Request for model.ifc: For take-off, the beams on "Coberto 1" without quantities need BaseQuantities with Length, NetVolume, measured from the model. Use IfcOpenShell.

First a look at what the model holds.

```python
import ifcopenshell
import ifcopenshell.util.element
import ifcopenshell.util.unit

model = ifcopenshell.open("model.ifc")
print(model.schema)
for unit_type in ("LENGTHUNIT", "AREAUNIT", "VOLUMEUNIT"):
    print(unit_type, ifcopenshell.util.unit.calculate_unit_scale(model, unit_type))
storey = next(s for s in model.by_type("IfcBuildingStorey") if s.Name == "Coberto 1")
beams = [e for e in ifcopenshell.util.element.get_decomposition(storey) if e.is_a("IfcBeam")]
for e in sorted(beams, key=lambda e: e.id()):
    print(e.id(), e.is_a(), e.Name, list(ifcopenshell.util.element.get_psets(e, qtos_only=True)), sep=" | ")
```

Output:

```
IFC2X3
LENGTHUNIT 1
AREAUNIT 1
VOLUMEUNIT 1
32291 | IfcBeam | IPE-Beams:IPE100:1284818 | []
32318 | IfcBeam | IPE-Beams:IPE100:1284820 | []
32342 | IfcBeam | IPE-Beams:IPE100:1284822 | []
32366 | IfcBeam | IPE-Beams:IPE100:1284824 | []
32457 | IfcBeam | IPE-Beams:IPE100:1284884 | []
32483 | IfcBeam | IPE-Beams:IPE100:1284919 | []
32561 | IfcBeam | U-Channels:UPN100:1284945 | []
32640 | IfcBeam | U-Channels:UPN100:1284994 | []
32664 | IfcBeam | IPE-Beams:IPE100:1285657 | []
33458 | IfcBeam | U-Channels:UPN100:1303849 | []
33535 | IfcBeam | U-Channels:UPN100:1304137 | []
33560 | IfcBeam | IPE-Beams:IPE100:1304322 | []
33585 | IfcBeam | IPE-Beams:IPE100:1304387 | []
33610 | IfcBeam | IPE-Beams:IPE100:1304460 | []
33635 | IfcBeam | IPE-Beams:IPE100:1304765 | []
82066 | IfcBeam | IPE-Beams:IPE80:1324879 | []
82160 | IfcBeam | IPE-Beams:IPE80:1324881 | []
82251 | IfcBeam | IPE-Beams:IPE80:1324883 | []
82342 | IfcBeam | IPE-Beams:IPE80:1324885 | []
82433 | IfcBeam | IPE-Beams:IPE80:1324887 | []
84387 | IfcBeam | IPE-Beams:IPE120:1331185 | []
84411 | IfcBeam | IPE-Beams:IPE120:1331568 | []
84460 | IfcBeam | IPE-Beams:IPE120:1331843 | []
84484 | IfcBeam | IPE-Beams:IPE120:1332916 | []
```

```python
import ifcopenshell
import ifcopenshell.api.pset
import ifcopenshell.geom
import ifcopenshell.util.element
import ifcopenshell.util.shape
import ifcopenshell.util.unit

model = ifcopenshell.open("model.ifc")
unit_scale = ifcopenshell.util.unit.calculate_unit_scale(model)
volume_scale = ifcopenshell.util.unit.calculate_unit_scale(model, "VOLUMEUNIT")
settings = ifcopenshell.geom.settings()

storey = next(s for s in model.by_type("IfcBuildingStorey") if s.Name == "Coberto 1")
beams = [e for e in ifcopenshell.util.element.get_decomposition(storey) if e.is_a("IfcBeam")]

for e in sorted(beams, key=lambda e: e.id()):
    if ifcopenshell.util.element.get_psets(e, qtos_only=True, should_inherit=False):
        continue
    # Geometry comes back in metres, in the element's own axes.
    shape = ifcopenshell.geom.create_shape(settings, e)
    values = {
        "Length": ifcopenshell.util.shape.get_max_xyz(shape.geometry) / unit_scale,
        "NetVolume": ifcopenshell.util.shape.get_volume(shape.geometry) / volume_scale,
    }
    qto = ifcopenshell.api.pset.add_qto(model, product=e, name="BaseQuantities")
    ifcopenshell.api.pset.edit_qto(model, qto=qto, properties=values)
    print(e.id(), {k: round(v, 3) for k, v in values.items()})

model.write("model_v2.ifc")
```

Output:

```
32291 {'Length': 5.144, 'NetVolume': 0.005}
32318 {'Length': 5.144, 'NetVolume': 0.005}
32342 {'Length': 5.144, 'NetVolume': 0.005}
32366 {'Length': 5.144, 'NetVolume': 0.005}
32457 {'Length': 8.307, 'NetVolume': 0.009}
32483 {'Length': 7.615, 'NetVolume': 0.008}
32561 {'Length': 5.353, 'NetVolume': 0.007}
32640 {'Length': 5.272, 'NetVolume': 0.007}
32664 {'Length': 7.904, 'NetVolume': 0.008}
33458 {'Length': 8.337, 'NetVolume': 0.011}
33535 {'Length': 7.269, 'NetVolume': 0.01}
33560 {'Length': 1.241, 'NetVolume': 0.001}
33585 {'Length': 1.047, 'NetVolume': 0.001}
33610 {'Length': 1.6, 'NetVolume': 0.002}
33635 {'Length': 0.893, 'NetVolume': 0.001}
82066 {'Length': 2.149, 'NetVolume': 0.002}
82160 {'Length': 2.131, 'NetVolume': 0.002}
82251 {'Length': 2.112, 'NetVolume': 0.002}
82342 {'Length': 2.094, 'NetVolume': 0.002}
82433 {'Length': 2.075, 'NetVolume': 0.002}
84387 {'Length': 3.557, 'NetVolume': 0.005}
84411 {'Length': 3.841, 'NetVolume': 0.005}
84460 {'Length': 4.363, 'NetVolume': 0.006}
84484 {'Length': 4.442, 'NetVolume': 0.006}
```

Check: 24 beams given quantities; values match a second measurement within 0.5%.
